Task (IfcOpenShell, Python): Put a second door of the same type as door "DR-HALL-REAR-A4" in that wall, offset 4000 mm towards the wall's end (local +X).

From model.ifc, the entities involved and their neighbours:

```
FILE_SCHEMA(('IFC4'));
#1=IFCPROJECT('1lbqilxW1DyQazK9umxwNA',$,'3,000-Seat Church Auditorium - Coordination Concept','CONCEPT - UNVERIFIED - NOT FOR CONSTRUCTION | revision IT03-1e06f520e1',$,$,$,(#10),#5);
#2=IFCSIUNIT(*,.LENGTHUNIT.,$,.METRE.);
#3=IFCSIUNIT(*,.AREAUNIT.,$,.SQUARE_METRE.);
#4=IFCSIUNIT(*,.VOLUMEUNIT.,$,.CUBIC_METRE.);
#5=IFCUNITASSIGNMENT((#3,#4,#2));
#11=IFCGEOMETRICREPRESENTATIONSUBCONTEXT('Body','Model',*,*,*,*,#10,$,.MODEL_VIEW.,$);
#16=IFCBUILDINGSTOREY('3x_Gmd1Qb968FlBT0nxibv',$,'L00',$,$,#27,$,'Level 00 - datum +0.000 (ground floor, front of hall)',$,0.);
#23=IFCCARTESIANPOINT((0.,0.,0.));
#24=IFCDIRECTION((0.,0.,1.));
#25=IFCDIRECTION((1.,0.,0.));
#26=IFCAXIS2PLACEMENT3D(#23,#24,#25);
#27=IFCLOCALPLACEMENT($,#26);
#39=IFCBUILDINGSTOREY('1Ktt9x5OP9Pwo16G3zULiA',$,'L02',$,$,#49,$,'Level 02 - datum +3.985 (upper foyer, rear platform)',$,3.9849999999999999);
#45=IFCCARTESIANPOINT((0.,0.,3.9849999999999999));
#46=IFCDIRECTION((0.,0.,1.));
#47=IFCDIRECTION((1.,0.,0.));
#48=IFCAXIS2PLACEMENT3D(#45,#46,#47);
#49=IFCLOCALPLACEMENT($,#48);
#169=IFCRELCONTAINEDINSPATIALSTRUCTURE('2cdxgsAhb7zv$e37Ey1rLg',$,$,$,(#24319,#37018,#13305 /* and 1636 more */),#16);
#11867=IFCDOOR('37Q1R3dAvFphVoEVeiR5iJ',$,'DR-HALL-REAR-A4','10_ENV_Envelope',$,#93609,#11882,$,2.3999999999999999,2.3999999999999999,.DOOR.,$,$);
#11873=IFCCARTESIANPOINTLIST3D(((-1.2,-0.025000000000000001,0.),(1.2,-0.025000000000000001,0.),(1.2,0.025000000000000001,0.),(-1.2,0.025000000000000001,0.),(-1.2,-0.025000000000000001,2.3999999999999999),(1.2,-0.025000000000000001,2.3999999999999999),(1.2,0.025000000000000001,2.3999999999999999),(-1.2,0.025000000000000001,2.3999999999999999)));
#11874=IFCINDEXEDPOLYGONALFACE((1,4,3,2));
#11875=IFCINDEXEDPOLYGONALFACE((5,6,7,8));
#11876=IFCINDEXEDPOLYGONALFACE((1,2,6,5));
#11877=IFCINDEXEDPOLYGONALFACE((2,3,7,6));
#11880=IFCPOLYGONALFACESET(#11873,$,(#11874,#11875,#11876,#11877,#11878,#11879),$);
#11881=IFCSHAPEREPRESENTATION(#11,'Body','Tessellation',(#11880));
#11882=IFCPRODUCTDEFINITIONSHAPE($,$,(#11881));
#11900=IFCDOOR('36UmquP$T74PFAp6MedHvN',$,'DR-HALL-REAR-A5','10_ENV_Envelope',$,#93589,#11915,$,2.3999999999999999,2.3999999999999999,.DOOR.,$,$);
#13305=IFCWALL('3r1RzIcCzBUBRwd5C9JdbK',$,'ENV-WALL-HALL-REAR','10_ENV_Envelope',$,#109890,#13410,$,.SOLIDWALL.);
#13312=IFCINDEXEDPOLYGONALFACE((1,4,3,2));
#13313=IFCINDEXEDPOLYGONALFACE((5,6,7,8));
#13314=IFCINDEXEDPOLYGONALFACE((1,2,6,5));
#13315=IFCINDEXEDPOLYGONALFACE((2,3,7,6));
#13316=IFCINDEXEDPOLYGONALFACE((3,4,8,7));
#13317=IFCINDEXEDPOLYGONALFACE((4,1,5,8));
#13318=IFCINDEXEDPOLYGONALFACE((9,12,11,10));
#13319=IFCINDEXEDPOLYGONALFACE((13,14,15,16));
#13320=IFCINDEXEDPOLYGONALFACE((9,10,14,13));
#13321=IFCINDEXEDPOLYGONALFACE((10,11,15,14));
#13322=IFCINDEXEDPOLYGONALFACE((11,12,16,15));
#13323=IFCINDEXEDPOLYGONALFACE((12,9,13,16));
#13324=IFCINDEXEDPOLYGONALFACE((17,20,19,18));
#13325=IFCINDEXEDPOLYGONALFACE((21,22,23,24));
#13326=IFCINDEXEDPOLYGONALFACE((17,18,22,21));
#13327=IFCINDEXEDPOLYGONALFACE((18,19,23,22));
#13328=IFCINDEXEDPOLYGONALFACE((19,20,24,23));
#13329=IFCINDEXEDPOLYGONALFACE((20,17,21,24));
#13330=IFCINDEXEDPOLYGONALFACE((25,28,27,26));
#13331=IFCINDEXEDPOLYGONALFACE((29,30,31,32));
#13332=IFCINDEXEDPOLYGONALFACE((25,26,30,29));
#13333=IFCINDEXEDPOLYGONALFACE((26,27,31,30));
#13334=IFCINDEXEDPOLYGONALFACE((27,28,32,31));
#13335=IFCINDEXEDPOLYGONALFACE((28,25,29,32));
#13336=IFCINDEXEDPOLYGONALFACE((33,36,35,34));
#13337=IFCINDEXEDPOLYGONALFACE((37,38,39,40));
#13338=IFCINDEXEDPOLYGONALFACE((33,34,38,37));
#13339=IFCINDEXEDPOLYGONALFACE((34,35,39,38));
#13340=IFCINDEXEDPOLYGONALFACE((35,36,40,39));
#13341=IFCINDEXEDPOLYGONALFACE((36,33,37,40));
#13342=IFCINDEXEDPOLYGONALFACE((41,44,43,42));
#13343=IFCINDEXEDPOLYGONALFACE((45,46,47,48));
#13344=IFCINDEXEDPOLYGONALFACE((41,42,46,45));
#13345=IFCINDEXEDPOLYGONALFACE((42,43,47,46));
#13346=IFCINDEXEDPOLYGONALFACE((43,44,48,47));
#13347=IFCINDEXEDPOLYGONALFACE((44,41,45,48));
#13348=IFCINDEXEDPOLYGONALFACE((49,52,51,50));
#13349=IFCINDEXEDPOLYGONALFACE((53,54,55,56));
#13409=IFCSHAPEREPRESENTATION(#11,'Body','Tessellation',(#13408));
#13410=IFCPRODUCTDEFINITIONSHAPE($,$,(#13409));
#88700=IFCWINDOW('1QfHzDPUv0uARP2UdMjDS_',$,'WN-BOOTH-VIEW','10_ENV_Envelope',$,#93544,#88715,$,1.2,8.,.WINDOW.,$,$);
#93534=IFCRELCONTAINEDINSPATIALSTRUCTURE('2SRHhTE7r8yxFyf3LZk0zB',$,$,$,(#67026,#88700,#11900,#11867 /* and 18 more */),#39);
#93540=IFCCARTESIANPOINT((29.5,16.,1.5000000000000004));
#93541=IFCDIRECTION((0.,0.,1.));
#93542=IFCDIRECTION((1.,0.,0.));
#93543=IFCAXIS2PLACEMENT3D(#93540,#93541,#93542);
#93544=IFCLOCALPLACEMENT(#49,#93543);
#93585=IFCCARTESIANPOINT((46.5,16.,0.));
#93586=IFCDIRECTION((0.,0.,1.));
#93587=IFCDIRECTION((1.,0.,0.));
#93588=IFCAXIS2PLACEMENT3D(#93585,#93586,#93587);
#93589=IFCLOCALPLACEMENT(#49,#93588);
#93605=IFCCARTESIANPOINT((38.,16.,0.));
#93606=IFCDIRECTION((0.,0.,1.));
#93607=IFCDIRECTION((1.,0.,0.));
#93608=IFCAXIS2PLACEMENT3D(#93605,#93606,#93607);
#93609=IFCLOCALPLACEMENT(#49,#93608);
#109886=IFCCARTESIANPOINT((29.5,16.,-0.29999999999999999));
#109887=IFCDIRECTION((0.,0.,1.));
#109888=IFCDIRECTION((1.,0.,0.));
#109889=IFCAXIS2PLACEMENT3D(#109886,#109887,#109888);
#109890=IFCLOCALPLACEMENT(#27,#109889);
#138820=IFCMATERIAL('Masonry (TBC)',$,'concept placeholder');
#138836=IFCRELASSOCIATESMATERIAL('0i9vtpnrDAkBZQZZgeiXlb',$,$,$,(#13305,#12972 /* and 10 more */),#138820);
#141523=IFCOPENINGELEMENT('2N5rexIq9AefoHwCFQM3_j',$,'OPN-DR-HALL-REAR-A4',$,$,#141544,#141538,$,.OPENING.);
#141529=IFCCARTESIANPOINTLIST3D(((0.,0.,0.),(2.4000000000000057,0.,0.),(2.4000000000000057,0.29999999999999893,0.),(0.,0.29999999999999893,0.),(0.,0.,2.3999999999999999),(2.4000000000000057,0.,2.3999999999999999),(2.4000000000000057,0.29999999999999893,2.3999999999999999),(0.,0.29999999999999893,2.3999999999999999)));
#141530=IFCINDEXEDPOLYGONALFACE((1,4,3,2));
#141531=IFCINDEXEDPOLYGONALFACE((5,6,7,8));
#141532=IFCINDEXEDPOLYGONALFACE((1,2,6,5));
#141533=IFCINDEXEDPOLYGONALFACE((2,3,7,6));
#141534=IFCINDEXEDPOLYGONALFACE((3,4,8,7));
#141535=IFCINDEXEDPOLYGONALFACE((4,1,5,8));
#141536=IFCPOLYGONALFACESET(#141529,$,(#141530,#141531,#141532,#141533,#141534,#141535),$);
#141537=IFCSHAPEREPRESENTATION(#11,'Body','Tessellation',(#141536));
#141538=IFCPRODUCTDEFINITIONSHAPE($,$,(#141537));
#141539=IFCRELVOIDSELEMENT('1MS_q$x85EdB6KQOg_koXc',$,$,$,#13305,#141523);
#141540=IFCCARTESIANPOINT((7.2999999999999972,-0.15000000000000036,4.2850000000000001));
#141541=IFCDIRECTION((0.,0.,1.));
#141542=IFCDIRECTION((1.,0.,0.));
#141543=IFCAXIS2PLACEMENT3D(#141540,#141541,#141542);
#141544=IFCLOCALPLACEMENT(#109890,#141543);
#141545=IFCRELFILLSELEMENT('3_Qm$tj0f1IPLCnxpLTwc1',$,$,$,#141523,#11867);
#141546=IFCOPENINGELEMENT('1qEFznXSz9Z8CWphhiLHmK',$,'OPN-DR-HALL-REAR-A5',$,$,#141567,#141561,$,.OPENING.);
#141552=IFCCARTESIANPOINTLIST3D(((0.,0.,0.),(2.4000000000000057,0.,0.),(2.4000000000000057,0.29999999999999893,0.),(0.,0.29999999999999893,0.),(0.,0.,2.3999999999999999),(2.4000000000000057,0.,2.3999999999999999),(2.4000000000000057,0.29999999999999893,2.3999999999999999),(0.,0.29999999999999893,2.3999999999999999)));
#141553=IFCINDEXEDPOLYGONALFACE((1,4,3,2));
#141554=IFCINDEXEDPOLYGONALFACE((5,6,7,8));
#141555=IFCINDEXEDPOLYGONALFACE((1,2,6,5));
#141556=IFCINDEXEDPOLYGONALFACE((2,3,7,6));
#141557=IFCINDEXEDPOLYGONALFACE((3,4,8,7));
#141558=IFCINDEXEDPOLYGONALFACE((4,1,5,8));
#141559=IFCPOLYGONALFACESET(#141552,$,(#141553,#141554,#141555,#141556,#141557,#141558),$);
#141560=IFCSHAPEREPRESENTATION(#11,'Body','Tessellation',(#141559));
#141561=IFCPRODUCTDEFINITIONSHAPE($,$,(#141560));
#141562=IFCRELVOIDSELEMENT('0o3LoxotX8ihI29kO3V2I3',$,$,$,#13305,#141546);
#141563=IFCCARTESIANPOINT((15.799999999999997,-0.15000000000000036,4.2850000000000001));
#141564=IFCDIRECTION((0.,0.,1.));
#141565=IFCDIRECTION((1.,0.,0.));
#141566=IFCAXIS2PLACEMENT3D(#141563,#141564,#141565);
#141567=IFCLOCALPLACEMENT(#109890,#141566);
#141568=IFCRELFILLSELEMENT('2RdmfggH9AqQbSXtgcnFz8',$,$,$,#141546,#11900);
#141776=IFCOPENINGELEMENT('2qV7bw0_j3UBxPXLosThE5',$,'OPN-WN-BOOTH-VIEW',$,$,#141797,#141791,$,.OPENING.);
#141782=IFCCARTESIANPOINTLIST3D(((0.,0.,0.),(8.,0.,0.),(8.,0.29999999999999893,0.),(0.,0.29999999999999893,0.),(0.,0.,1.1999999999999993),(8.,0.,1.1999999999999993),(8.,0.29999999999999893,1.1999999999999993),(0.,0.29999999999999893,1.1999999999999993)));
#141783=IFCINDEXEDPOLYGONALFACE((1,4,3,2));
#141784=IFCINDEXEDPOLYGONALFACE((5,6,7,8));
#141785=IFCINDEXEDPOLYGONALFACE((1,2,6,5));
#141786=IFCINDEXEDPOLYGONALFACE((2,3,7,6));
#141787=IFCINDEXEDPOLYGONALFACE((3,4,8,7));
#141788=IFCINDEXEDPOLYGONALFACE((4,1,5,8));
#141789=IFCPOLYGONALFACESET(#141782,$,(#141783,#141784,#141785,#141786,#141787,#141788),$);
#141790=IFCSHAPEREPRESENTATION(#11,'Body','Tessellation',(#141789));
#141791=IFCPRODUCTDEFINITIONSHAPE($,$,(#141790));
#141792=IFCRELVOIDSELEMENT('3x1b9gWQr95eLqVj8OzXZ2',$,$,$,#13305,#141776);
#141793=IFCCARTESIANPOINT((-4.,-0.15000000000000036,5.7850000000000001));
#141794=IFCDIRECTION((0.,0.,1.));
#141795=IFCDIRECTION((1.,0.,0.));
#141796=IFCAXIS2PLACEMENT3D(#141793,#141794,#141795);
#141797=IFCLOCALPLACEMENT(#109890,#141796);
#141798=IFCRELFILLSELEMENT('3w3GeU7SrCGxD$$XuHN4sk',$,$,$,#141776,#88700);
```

```python
import ifcopenshell
import ifcopenshell.api.feature
import ifcopenshell.api.geometry
import ifcopenshell.api.root
import ifcopenshell.geom
import ifcopenshell.util.element
import ifcopenshell.util.placement
import ifcopenshell.util.shape

model = ifcopenshell.open("model.ifc")
settings = ifcopenshell.geom.settings()


def volume(element):
    """Net volume in cubic metres, openings subtracted."""
    shape = ifcopenshell.geom.create_shape(settings, element)
    return ifcopenshell.util.shape.get_volume(shape.geometry)


door = model.by_guid("37Q1R3dAvFphVoEVeiR5iJ")
opening = door.FillsVoids[0].RelatingOpeningElement
wall = opening.VoidsElements[0].RelatingBuildingElement
before = volume(wall)
shift = ifcopenshell.util.placement.get_local_placement(wall.ObjectPlacement)[:3, 0] * 4.0

# copy_class copies the void relationship, type, container and properties, but no geometry.
new_opening = ifcopenshell.api.root.copy_class(model, product=opening)
new_opening.Representation = ifcopenshell.util.element.copy_deep(
    model, opening.Representation, exclude=["IfcGeometricRepresentationContext", "IfcRepresentationMap"]
)
new_door = ifcopenshell.api.root.copy_class(model, product=door)
new_door.Representation = ifcopenshell.util.element.copy_deep(
    model, door.Representation, exclude=["IfcGeometricRepresentationContext", "IfcRepresentationMap"]
)
ifcopenshell.api.feature.add_filling(model, opening=new_opening, element=new_door)

for old, new in ((opening, new_opening), (door, new_door)):
    matrix = ifcopenshell.util.placement.get_local_placement(old.ObjectPlacement)
    matrix[:3, 3] += shift
    ifcopenshell.api.geometry.edit_object_placement(model, product=new, matrix=matrix, is_si=False)

after = volume(wall)

print(f"wall volume {before:.3f} -> {after:.3f} m3")

model.write("model_rev.ifc")
```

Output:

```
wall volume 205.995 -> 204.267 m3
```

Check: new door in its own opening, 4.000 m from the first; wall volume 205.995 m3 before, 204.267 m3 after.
